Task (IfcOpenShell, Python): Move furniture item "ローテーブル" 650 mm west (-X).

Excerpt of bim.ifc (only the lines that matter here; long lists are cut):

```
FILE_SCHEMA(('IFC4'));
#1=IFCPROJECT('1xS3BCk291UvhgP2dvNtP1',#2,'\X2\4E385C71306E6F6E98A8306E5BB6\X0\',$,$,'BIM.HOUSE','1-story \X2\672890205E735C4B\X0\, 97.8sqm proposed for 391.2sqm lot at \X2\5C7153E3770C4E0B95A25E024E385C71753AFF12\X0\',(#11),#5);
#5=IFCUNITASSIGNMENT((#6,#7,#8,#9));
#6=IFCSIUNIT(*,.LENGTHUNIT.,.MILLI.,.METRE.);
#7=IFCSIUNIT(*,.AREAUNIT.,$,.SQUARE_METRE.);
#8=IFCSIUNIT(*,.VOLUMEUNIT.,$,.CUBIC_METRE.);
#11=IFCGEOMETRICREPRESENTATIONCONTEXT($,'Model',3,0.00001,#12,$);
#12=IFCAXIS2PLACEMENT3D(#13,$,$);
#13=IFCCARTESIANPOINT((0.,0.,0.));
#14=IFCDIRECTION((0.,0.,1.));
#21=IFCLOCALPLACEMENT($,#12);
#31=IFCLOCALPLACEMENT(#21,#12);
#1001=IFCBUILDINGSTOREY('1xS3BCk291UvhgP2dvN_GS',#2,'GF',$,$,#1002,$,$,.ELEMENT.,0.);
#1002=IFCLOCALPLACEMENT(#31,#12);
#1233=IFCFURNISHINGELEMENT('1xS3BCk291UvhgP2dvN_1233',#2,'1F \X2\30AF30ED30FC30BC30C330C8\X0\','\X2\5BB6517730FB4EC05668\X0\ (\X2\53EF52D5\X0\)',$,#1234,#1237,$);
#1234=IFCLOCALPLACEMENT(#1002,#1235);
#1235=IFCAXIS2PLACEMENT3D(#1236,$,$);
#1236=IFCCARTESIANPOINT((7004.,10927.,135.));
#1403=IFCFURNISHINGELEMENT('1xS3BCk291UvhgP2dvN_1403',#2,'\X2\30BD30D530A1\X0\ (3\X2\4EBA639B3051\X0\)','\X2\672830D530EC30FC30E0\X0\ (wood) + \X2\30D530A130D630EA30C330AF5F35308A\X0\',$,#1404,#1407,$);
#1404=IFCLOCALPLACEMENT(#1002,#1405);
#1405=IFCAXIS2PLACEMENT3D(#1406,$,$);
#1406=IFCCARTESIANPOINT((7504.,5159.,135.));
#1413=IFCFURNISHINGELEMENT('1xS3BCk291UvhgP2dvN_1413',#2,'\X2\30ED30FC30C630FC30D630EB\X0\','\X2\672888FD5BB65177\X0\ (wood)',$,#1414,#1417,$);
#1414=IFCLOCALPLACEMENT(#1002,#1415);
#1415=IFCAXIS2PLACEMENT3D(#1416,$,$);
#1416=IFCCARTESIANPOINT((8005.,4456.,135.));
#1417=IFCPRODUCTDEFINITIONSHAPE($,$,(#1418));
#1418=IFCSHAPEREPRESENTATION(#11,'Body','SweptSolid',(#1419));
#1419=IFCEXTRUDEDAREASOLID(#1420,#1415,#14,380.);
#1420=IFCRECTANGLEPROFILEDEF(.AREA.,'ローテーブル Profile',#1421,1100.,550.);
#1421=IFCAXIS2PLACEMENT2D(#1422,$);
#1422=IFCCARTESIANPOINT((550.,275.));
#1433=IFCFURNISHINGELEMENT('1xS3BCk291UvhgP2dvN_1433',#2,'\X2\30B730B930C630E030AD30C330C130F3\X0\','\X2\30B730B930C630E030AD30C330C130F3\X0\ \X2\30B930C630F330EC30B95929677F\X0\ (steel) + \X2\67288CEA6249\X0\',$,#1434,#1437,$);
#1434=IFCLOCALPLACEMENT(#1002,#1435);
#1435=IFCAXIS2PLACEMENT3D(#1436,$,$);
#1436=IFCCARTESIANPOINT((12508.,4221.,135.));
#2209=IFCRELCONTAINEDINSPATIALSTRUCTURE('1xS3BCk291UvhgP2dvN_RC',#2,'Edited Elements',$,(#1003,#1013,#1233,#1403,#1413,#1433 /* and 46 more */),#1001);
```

```python
import ifcopenshell
import ifcopenshell.api.geometry
import ifcopenshell.util.placement
import ifcopenshell.util.unit

model = ifcopenshell.open("bim.ifc")
unit_scale = ifcopenshell.util.unit.calculate_unit_scale(model)

item = model.by_guid("1xS3BCk291UvhgP2dvN_1413")
matrix = ifcopenshell.util.placement.get_local_placement(item.ObjectPlacement)
matrix[0, 3] -= 0.65 / unit_scale
ifcopenshell.api.geometry.edit_object_placement(model, product=item, matrix=matrix, is_si=False)

print(ifcopenshell.util.placement.get_local_placement(item.ObjectPlacement).round(3) + 0.0)

model.write("bim_edited.ifc")
```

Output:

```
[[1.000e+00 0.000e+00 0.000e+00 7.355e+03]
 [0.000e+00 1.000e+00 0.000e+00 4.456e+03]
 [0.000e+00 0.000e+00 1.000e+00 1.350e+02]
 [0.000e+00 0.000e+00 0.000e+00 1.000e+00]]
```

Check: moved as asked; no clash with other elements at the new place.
